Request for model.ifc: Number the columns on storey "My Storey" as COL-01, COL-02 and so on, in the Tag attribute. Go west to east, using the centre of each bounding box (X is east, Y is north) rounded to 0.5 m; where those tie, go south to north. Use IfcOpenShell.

First a look at what the model holds.

```python
import ifcopenshell
import ifcopenshell.util.element
import ifcopenshell.util.placement

model = ifcopenshell.open("model.ifc")
print(model.schema)
storey = next(s for s in model.by_type("IfcBuildingStorey") if s.Name == "My Storey")
columns = [e for e in ifcopenshell.util.element.get_decomposition(storey) if e.is_a("IfcColumn")]
for e in sorted(columns, key=lambda e: e.id()):
    origin = ifcopenshell.util.placement.get_local_placement(e.ObjectPlacement)[:3, 3]
    print(e.id(), e.Tag, e.Name, origin.round(2) + 0.0, sep=" | ")
```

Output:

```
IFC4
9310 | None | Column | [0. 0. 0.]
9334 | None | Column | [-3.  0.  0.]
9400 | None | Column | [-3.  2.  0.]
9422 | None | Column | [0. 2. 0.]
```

```python
import ifcopenshell
import ifcopenshell.geom
import ifcopenshell.util.element
import ifcopenshell.util.shape

model = ifcopenshell.open("model.ifc")
settings = ifcopenshell.geom.settings()
settings.set("use-world-coords", True)


def centre(element):
    shape = ifcopenshell.geom.create_shape(settings, element)
    return ifcopenshell.util.shape.get_bbox_centroid(shape.geometry)


storey = next(s for s in model.by_type("IfcBuildingStorey") if s.Name == "My Storey")
columns = [e for e in ifcopenshell.util.element.get_decomposition(storey) if e.is_a("IfcColumn")]

# Insertion points can sit at a corner or the storey origin, so sort by the geometry (in metres).
centres = {e: centre(e) for e in columns}
columns.sort(key=lambda e: (round(centres[e][0] / 0.5), centres[e][1]))

for i, e in enumerate(columns, start=1):
    number = f"COL-{i:02d}"
    e.Tag = number
    print(e.id(), number)

model.write("model_updated.ifc")
```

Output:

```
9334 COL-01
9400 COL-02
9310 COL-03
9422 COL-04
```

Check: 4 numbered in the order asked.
